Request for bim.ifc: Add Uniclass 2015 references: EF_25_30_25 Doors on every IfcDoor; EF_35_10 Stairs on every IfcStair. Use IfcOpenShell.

First a look at what the model holds.

```python
import ifcopenshell

model = ifcopenshell.open("bim.ifc")
print(model.schema)
print("classifications:", [c.Name for c in model.by_type("IfcClassification")])
for ifc_class in ("IfcDoor", "IfcRoof", "IfcStair", "IfcWall", "IfcWindow"):
    print(ifc_class, len(model.by_type(ifc_class)))
```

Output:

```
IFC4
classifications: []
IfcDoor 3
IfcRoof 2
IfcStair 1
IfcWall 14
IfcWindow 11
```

```python
import ifcopenshell
import ifcopenshell.api.classification

model = ifcopenshell.open("bim.ifc")

system = ifcopenshell.api.classification.add_classification(model, classification="Uniclass 2015")

codes = {
    "IfcDoor": ("EF_25_30_25", "Doors"),
    "IfcStair": ("EF_35_10", "Stairs"),
}
for ifc_class, (code, name) in codes.items():
    products = model.by_type(ifc_class)
    ifcopenshell.api.classification.add_reference(
        model, products=products, classification=system, identification=code, name=name
    )
    print(code, len(products))

model.write("bim_updated.ifc")
```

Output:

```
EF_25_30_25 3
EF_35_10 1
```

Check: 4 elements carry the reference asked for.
